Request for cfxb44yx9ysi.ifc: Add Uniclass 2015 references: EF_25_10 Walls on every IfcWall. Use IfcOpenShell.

First a look at what the model holds.

```python
import ifcopenshell

model = ifcopenshell.open("cfxb44yx9ysi.ifc")
print(model.schema)
print("classifications:", [c.Name for c in model.by_type("IfcClassification")])
for ifc_class in ("IfcDoor", "IfcRoof", "IfcStair", "IfcWall", "IfcWindow"):
    print(ifc_class, len(model.by_type(ifc_class)))
```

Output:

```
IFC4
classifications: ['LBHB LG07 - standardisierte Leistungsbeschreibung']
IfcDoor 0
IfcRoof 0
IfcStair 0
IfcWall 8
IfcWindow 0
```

```python
import ifcopenshell
import ifcopenshell.api.classification

model = ifcopenshell.open("cfxb44yx9ysi.ifc")

system = ifcopenshell.api.classification.add_classification(model, classification="Uniclass 2015")

codes = {
    "IfcWall": ("EF_25_10", "Walls"),
}
for ifc_class, (code, name) in codes.items():
    products = model.by_type(ifc_class)
    ifcopenshell.api.classification.add_reference(
        model, products=products, classification=system, identification=code, name=name
    )
    print(code, len(products))

model.write("cfxb44yx9ysi-out.ifc")
```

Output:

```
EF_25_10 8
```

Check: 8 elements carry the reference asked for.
